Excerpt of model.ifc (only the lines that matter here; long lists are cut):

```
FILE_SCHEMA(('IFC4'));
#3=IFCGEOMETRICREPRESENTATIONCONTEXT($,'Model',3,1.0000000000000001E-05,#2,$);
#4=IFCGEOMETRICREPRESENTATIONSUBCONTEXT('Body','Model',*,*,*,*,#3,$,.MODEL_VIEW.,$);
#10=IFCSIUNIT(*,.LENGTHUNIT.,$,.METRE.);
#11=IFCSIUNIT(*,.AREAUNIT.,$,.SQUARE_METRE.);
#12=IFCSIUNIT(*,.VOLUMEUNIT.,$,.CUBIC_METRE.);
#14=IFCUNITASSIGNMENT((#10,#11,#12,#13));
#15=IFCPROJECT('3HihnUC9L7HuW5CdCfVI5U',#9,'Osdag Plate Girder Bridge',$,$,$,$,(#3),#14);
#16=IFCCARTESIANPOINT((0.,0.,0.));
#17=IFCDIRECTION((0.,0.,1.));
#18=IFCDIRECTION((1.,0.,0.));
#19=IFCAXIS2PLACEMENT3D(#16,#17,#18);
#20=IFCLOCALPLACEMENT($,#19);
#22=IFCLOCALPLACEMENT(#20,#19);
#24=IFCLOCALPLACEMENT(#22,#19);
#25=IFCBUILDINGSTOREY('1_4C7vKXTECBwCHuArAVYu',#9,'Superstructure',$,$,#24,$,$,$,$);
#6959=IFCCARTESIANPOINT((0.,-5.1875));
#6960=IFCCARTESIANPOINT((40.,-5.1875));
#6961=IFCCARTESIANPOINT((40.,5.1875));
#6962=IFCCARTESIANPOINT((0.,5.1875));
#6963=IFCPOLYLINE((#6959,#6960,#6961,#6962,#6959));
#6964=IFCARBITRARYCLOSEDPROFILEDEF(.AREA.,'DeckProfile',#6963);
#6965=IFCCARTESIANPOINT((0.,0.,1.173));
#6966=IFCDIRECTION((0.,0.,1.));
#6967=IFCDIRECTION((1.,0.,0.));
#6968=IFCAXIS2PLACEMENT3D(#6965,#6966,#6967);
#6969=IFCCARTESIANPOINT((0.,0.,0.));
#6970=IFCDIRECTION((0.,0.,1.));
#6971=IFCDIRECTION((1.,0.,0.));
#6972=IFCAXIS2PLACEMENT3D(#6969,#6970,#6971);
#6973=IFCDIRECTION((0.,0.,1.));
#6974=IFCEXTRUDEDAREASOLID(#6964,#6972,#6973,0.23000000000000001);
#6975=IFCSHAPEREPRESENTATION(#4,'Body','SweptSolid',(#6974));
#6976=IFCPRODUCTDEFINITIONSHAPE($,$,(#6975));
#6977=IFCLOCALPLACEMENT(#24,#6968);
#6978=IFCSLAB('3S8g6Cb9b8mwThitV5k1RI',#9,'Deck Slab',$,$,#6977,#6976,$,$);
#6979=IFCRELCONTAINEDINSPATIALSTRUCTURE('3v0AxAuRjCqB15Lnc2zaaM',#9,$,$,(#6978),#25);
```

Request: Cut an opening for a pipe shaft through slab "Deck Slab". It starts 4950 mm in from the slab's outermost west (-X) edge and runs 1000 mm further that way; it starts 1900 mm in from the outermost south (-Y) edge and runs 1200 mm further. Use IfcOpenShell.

```python
import numpy as np
import ifcopenshell
import ifcopenshell.api.feature
import ifcopenshell.api.geometry
import ifcopenshell.api.root
import ifcopenshell.geom
import ifcopenshell.util.placement
import ifcopenshell.util.representation
import ifcopenshell.util.shape
import ifcopenshell.util.unit

model = ifcopenshell.open("model.ifc")
unit_scale = ifcopenshell.util.unit.calculate_unit_scale(model)
settings = ifcopenshell.geom.settings()


def volume(element):
    """Net volume in cubic metres, openings subtracted."""
    shape = ifcopenshell.geom.create_shape(settings, element)
    return ifcopenshell.util.shape.get_volume(shape.geometry)


slab = model.by_id(6978)
before = volume(slab)

# Extent in the slab's own axes, in metres. The edges named are its -X and -Y sides.
slab_shape = ifcopenshell.geom.create_shape(settings, slab)
vertices = ifcopenshell.util.shape.get_vertices(slab_shape.geometry)
x_min, y_min, bottom = vertices.min(axis=0)
top = vertices[:, 2].max()

opening = ifcopenshell.api.root.create_entity(model, ifc_class="IfcOpeningElement", name="Pipe shaft opening", predefined_type="OPENING")
context = ifcopenshell.util.representation.get_context(model, "Model", "Body", "MODEL_VIEW")
width, depth = 1, 1.2
outline = [(0.0, 0.0), (width, 0.0), (width, depth), (0.0, depth), (0.0, 0.0)]
# Overshoot both faces by 50 mm so the cut is clean.
shape = ifcopenshell.api.geometry.add_slab_representation(
    model, context=context, depth=top - bottom + 0.1, polyline=outline
)
ifcopenshell.api.geometry.assign_representation(model, product=opening, representation=shape)

matrix = ifcopenshell.util.placement.get_local_placement(slab.ObjectPlacement)
matrix[:, 3] = matrix @ np.append(np.array([x_min + 4.95, y_min + 1.9, bottom - 0.05]) / unit_scale, 1.0)
ifcopenshell.api.geometry.edit_object_placement(model, product=opening, matrix=matrix, is_si=False)
ifcopenshell.api.feature.add_feature(model, feature=opening, element=slab)

after = volume(slab)

print(f"slab volume {before:.3f} -> {after:.3f} m3")

model.write("model_updated.ifc")
```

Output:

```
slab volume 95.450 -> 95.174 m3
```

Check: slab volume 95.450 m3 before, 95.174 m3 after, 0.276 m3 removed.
